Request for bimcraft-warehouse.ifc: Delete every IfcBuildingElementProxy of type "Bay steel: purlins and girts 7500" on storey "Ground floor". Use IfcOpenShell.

First a look at what the model holds.

```python
import ifcopenshell
import ifcopenshell.util.element

model = ifcopenshell.open("bimcraft-warehouse.ifc")
print(model.schema)
storey = next(s for s in model.by_type("IfcBuildingStorey") if s.Name == "Ground floor")
proxies = [e for e in ifcopenshell.util.element.get_decomposition(storey) if e.is_a("IfcBuildingElementProxy")]
seen = {}
for e in proxies:
    element_type = ifcopenshell.util.element.get_type(e)
    name = element_type.Name if element_type not in (None, e) else None
    seen[name] = seen.get(name, 0) + 1
for name, count in sorted(seen.items(), key=str):
    print(count, "x", name)
```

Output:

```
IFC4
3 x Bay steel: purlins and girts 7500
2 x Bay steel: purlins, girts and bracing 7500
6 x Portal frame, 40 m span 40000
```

```python
import ifcopenshell
import ifcopenshell.api.root
import ifcopenshell.util.element

model = ifcopenshell.open("bimcraft-warehouse.ifc")

storey = next(s for s in model.by_type("IfcBuildingStorey") if s.Name == "Ground floor")
proxies = [e for e in ifcopenshell.util.element.get_decomposition(storey) if e.is_a("IfcBuildingElementProxy")]
targets = [e for e in proxies if (t := ifcopenshell.util.element.get_type(e)) not in (None, e) and t.Name == "Bay steel: purlins and girts 7500"]

for e in targets:
    ifcopenshell.api.root.remove_product(model, product=e)
print(len(targets), "removed")

model.write("bimcraft-warehouse_v2.ifc")
```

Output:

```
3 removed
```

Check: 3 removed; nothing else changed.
